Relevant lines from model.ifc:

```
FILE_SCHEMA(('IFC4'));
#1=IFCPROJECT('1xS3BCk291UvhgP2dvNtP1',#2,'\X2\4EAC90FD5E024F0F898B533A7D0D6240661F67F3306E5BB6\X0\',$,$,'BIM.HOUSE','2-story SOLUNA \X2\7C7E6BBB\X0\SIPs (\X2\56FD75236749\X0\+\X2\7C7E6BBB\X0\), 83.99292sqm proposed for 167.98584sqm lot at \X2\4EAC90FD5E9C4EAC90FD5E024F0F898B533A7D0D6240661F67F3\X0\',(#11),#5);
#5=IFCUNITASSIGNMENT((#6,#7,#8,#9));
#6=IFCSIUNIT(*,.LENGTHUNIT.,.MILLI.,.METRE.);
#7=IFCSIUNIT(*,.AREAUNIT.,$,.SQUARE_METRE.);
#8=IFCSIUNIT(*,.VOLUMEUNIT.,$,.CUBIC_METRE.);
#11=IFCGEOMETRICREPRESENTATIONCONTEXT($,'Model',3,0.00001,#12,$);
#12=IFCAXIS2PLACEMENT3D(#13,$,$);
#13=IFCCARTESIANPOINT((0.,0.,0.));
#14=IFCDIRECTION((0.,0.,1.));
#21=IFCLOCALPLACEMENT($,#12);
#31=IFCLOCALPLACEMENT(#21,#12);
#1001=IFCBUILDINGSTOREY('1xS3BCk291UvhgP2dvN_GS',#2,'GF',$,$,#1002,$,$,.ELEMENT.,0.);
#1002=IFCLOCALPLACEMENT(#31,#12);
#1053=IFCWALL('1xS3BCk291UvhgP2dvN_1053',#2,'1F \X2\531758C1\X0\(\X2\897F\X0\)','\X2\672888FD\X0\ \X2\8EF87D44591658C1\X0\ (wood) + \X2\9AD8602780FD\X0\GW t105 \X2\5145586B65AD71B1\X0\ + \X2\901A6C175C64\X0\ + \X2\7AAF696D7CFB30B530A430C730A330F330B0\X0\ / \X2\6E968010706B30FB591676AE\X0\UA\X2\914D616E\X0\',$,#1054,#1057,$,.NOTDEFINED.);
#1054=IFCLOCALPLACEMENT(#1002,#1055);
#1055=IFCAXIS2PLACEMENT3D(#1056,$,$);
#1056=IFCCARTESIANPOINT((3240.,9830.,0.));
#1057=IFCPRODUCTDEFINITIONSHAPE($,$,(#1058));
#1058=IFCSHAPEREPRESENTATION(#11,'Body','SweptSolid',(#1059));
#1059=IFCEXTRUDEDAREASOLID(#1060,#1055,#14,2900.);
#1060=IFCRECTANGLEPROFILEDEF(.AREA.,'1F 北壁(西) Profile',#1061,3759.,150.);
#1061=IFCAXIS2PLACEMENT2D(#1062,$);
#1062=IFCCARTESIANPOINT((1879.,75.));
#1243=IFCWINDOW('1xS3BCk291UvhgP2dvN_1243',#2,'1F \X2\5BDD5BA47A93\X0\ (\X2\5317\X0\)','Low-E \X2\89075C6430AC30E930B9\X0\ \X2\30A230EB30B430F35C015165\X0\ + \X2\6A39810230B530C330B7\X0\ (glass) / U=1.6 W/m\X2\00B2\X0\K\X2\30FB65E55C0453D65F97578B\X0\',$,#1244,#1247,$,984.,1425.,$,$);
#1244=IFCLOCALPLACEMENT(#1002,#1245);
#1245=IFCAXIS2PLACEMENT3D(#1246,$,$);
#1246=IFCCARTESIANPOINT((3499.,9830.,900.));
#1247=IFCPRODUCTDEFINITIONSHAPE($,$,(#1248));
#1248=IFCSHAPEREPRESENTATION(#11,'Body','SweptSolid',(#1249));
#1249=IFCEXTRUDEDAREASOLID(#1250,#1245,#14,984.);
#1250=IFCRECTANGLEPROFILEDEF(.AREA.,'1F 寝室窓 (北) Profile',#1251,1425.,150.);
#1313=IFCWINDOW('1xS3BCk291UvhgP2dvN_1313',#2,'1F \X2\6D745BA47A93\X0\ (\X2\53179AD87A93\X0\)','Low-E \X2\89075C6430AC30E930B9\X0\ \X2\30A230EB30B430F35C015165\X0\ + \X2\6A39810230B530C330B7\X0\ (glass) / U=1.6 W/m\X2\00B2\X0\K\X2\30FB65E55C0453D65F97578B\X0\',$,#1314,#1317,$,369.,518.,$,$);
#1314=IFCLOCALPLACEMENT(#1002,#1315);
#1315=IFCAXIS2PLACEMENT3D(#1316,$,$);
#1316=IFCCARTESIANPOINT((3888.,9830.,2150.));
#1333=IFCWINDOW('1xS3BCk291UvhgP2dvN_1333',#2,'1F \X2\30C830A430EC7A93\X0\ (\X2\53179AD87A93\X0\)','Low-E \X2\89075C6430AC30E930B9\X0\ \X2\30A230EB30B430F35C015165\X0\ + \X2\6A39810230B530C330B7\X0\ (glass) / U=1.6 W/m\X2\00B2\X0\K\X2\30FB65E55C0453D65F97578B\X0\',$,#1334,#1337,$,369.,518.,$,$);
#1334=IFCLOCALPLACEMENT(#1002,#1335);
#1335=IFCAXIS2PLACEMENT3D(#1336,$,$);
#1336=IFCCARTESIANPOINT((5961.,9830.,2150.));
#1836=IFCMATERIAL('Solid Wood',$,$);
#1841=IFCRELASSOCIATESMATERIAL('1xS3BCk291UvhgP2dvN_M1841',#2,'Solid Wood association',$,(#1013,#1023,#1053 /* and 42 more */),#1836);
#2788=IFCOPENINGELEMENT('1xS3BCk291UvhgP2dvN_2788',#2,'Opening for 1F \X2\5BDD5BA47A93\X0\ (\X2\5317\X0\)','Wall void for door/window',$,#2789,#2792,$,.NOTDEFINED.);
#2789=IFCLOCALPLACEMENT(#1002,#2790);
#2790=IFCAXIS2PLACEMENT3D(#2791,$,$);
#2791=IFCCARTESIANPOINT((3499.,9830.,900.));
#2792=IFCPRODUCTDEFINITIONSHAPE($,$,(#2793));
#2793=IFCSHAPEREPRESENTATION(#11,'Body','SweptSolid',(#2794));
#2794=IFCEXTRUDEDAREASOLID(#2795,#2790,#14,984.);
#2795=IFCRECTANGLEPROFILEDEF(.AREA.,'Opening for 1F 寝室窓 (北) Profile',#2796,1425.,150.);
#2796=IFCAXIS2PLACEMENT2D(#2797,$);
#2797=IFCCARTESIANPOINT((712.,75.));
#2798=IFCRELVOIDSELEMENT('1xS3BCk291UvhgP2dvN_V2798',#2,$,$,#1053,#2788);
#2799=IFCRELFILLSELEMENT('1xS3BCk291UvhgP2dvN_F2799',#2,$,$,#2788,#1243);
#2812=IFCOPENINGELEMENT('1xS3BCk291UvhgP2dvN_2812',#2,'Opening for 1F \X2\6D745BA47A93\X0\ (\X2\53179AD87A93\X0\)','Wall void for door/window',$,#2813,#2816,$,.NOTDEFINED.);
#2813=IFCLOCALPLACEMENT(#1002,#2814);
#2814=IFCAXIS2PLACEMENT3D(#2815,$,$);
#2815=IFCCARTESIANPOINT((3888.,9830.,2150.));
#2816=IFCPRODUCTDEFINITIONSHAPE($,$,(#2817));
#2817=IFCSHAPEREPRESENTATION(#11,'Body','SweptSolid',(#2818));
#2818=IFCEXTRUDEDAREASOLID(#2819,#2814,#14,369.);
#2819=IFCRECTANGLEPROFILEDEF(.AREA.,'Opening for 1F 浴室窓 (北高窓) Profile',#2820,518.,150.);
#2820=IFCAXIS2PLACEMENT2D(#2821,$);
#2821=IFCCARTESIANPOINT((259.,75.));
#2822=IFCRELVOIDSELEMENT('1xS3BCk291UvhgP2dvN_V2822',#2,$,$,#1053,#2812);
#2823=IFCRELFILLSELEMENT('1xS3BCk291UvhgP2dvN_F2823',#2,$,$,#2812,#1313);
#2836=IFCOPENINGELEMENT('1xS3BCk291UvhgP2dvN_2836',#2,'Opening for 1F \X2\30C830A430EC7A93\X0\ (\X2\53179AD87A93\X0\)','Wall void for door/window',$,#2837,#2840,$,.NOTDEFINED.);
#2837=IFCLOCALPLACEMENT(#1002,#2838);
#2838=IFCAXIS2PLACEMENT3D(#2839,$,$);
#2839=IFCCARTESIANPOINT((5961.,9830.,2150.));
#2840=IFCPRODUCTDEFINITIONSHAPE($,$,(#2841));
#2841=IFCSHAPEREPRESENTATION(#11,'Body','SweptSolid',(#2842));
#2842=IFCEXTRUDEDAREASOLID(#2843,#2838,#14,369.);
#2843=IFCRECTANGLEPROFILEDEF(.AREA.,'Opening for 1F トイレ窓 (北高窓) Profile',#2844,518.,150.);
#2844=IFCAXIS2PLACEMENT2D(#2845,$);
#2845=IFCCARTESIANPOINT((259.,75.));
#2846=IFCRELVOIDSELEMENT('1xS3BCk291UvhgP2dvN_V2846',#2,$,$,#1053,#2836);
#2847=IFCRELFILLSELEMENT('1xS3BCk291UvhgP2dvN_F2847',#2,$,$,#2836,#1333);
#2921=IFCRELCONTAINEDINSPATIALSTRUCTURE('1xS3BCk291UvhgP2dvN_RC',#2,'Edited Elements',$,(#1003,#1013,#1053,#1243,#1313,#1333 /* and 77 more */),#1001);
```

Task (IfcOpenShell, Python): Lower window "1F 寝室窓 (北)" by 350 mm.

```python
import numpy as np
import ifcopenshell
import ifcopenshell.api.geometry
import ifcopenshell.util.placement
import ifcopenshell.util.unit

model = ifcopenshell.open("model.ifc")
unit_scale = ifcopenshell.util.unit.calculate_unit_scale(model)

window = model.by_guid("1xS3BCk291UvhgP2dvN_1243")
opening = window.FillsVoids[0].RelatingOpeningElement
dz = -0.35 / unit_scale

shift = np.array([0.0, 0.0, dz])
# The window is not placed relative to its opening, so move both.
for product in (opening, window):
    matrix = ifcopenshell.util.placement.get_local_placement(product.ObjectPlacement)
    matrix[:3, 3] += shift
    ifcopenshell.api.geometry.edit_object_placement(model, product=product, matrix=matrix, is_si=False)

print(f"moved by {dz * unit_scale:+.3f} m")

model.write("model_edited.ifc")
```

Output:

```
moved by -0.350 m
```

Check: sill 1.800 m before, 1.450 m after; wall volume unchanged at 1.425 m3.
